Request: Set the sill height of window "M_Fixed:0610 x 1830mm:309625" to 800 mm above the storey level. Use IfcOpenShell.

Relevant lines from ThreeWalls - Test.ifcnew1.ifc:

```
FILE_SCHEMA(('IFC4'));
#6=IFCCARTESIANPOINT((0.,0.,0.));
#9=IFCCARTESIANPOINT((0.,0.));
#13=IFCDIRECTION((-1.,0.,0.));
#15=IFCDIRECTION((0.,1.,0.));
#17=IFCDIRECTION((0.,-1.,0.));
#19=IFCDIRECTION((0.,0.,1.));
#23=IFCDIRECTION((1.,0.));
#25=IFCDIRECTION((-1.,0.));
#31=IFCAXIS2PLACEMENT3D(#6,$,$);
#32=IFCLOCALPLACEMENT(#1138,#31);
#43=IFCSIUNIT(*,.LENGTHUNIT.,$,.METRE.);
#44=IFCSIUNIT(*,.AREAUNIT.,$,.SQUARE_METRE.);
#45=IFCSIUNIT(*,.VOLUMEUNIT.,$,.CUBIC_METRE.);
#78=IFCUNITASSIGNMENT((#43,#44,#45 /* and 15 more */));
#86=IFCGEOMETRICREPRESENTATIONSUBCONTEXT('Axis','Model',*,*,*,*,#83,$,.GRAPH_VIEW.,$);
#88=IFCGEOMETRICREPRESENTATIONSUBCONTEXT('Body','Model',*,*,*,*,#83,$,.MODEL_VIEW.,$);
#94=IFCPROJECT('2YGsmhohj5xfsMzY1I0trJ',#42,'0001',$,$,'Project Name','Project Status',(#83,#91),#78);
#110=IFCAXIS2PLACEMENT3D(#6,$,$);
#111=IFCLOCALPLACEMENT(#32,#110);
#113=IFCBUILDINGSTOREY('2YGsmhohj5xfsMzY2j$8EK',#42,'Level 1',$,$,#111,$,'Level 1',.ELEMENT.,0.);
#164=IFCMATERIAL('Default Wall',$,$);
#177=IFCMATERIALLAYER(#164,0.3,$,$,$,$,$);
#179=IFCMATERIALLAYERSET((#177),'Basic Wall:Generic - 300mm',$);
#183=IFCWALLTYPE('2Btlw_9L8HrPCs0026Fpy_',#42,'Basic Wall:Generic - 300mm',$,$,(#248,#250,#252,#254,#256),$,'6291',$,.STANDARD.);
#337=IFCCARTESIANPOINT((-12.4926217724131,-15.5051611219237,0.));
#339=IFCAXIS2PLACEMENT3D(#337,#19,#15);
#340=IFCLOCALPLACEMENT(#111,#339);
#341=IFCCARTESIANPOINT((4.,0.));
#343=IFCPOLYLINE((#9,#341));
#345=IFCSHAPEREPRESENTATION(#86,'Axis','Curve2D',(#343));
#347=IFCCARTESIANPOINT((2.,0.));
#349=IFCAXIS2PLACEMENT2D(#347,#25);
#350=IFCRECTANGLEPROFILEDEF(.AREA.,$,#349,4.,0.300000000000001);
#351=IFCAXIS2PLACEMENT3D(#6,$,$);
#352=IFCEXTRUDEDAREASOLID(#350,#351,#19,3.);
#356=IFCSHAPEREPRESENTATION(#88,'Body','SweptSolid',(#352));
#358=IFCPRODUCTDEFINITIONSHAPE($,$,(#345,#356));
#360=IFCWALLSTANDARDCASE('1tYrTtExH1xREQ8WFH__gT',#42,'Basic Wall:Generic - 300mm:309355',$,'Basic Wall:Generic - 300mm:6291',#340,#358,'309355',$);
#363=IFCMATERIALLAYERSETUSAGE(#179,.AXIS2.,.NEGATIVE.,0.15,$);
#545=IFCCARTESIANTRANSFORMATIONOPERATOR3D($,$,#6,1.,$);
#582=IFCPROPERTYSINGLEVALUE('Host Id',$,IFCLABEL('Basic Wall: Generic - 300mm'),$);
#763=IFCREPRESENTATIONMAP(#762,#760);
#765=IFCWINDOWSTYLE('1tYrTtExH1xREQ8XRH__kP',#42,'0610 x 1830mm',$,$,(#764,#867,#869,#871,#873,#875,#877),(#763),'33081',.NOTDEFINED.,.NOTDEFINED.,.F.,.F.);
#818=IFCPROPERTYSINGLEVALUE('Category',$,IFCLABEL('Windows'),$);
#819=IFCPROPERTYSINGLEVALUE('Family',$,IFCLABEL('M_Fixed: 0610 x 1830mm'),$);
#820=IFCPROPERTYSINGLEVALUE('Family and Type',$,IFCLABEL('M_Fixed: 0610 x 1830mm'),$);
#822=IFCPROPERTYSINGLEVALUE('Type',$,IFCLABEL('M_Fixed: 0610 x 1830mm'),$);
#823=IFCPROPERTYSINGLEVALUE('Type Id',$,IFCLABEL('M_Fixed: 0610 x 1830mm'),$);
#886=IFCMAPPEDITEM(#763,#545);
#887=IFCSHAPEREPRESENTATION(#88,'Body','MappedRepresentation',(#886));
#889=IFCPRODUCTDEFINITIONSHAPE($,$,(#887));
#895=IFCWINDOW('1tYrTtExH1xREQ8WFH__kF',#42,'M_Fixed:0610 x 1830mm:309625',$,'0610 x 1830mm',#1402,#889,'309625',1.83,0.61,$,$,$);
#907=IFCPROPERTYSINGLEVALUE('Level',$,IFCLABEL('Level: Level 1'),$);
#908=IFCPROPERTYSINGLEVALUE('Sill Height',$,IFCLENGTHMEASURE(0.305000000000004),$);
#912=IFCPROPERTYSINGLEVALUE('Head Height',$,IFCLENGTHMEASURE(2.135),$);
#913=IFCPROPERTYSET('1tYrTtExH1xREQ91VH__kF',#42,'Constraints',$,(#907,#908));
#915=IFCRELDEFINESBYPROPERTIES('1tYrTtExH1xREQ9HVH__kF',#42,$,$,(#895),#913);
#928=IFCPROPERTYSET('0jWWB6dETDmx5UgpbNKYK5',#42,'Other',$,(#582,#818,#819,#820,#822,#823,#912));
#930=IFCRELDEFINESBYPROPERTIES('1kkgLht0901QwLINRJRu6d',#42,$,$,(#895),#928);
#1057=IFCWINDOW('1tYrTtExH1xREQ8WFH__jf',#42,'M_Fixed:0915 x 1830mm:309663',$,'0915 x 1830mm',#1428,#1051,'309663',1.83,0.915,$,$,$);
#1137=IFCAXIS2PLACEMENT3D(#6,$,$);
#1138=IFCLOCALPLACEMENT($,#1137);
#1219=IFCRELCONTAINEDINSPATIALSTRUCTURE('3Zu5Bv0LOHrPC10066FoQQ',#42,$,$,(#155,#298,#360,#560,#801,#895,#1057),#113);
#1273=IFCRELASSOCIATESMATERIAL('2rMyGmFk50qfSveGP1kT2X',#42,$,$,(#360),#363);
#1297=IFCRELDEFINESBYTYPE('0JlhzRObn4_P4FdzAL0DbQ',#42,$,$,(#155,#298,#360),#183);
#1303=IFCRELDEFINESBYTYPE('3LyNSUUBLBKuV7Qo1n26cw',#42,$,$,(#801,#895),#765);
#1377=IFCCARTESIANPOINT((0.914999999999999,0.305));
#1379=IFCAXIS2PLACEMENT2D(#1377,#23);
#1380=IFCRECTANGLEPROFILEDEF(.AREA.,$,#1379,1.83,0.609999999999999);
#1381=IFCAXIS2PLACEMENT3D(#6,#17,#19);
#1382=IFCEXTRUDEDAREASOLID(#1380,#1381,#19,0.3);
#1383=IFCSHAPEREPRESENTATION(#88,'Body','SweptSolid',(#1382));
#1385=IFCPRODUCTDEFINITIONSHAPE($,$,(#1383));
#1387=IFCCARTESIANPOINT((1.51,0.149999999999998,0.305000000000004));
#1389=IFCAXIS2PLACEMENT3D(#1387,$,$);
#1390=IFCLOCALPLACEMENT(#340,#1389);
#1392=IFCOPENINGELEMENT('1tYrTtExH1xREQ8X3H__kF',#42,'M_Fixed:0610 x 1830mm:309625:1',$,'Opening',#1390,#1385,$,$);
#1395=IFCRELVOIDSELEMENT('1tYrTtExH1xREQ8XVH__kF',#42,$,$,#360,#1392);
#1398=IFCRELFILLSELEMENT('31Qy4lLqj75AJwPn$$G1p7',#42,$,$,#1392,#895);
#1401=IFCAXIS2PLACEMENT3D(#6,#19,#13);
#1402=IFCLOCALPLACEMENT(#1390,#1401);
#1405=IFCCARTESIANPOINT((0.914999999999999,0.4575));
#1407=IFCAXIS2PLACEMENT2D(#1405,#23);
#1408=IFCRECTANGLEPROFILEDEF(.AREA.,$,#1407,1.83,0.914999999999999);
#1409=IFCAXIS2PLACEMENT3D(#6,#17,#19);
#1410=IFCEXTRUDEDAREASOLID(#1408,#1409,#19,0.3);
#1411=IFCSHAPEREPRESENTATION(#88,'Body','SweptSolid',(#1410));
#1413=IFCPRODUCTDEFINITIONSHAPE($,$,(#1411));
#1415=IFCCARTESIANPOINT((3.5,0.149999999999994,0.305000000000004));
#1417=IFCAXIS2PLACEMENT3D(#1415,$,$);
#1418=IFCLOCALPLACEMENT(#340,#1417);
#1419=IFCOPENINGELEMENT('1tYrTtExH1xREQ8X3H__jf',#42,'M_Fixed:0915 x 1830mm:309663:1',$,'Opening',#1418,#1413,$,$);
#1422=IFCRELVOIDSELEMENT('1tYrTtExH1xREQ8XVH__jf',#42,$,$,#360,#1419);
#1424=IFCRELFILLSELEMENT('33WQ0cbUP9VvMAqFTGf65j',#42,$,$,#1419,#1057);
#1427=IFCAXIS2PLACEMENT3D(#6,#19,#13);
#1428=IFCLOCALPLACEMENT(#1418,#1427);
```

```python
import numpy as np
import ifcopenshell
import ifcopenshell.api.geometry
import ifcopenshell.api.pset
import ifcopenshell.geom
import ifcopenshell.util.element
import ifcopenshell.util.placement
import ifcopenshell.util.shape
import ifcopenshell.util.unit

model = ifcopenshell.open("ThreeWalls - Test.ifcnew1.ifc")
unit_scale = ifcopenshell.util.unit.calculate_unit_scale(model)

window = model.by_guid("1tYrTtExH1xREQ8WFH__kF")
opening = window.FillsVoids[0].RelatingOpeningElement
storey = ifcopenshell.util.element.get_container(window, ifc_class="IfcBuildingStorey")
level = ifcopenshell.util.placement.get_local_placement(storey.ObjectPlacement)[2, 3]

# The opening's origin need not be at the sill, so measure its lowest point.
shape = ifcopenshell.geom.create_shape(ifcopenshell.geom.settings(), opening)
bottom = ifcopenshell.util.shape.get_shape_bottom_elevation(shape, shape.geometry) / unit_scale
dz = level + 0.8 - bottom

shift = np.array([0.0, 0.0, dz])
# The window is placed relative to its opening, so it follows when the opening moves.
matrix = ifcopenshell.util.placement.get_local_placement(opening.ObjectPlacement)
matrix[:3, 3] += shift
ifcopenshell.api.geometry.edit_object_placement(
    model, product=opening, matrix=matrix, is_si=False, should_transform_children=True
)

# Keep the stored heights in step.
pset = model.by_id(ifcopenshell.util.element.get_pset(window, "Constraints", should_inherit=False)["id"])
ifcopenshell.api.pset.edit_pset(model, pset=pset, properties={
    "Sill Height": model.create_entity("IfcLengthMeasure", ifcopenshell.util.element.get_pset(window, "Constraints", "Sill Height") + dz),
})
pset = model.by_id(ifcopenshell.util.element.get_pset(window, "Other", should_inherit=False)["id"])
ifcopenshell.api.pset.edit_pset(model, pset=pset, properties={
    "Head Height": model.create_entity("IfcLengthMeasure", ifcopenshell.util.element.get_pset(window, "Other", "Head Height") + dz),
})

print(f"moved by {dz * unit_scale:+.3f} m")

model.write("ThreeWalls - Test.ifcnew1_v2.ifc")
```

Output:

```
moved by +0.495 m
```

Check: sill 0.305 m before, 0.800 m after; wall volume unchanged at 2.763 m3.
